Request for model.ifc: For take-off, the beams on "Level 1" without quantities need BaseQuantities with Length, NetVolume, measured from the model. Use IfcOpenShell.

First a look at what the model holds.

```python
import ifcopenshell
import ifcopenshell.util.element
import ifcopenshell.util.unit

model = ifcopenshell.open("model.ifc")
print(model.schema)
for unit_type in ("LENGTHUNIT", "AREAUNIT", "VOLUMEUNIT"):
    print(unit_type, ifcopenshell.util.unit.calculate_unit_scale(model, unit_type))
storey = next(s for s in model.by_type("IfcBuildingStorey") if s.Name == "Level 1")
beams = [e for e in ifcopenshell.util.element.get_decomposition(storey) if e.is_a("IfcBeam")]
for e in sorted(beams, key=lambda e: e.id()):
    print(e.id(), e.is_a(), e.Name, list(ifcopenshell.util.element.get_psets(e, qtos_only=True)), sep=" | ")
```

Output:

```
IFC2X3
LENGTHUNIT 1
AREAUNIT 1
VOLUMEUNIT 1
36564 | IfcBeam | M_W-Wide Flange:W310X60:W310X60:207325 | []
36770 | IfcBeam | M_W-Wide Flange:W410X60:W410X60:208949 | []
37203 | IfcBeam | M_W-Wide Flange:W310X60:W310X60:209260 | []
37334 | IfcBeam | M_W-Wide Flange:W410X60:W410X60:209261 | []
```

```python
import ifcopenshell
import ifcopenshell.api.pset
import ifcopenshell.geom
import ifcopenshell.util.element
import ifcopenshell.util.shape
import ifcopenshell.util.unit

model = ifcopenshell.open("model.ifc")
unit_scale = ifcopenshell.util.unit.calculate_unit_scale(model)
volume_scale = ifcopenshell.util.unit.calculate_unit_scale(model, "VOLUMEUNIT")
settings = ifcopenshell.geom.settings()

storey = next(s for s in model.by_type("IfcBuildingStorey") if s.Name == "Level 1")
beams = [e for e in ifcopenshell.util.element.get_decomposition(storey) if e.is_a("IfcBeam")]

for e in sorted(beams, key=lambda e: e.id()):
    if ifcopenshell.util.element.get_psets(e, qtos_only=True, should_inherit=False):
        continue
    # Geometry comes back in metres, in the element's own axes.
    shape = ifcopenshell.geom.create_shape(settings, e)
    values = {
        "Length": ifcopenshell.util.shape.get_max_xyz(shape.geometry) / unit_scale,
        "NetVolume": ifcopenshell.util.shape.get_volume(shape.geometry) / volume_scale,
    }
    qto = ifcopenshell.api.pset.add_qto(model, product=e, name="BaseQuantities")
    ifcopenshell.api.pset.edit_qto(model, qto=qto, properties=values)
    print(e.id(), {k: round(v, 3) for k, v in values.items()})

model.write("model-out.ifc")
```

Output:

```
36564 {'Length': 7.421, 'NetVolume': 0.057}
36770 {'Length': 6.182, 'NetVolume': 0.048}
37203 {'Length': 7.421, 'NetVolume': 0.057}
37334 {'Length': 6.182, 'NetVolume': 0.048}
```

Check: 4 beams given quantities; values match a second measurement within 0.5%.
